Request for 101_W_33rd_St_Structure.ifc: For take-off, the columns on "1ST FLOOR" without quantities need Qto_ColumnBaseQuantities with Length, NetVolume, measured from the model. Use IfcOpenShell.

First a look at what the model holds.

```python
import ifcopenshell
import ifcopenshell.util.element
import ifcopenshell.util.unit

model = ifcopenshell.open("101_W_33rd_St_Structure.ifc")
print(model.schema)
for unit_type in ("LENGTHUNIT", "AREAUNIT", "VOLUMEUNIT"):
    print(unit_type, ifcopenshell.util.unit.calculate_unit_scale(model, unit_type))
storey = next(s for s in model.by_type("IfcBuildingStorey") if s.Name == "1ST FLOOR")
columns = [e for e in ifcopenshell.util.element.get_decomposition(storey) if e.is_a("IfcColumn")]
for e in sorted(columns, key=lambda e: e.id()):
    print(e.id(), e.is_a(), e.Name, list(ifcopenshell.util.element.get_psets(e, qtos_only=True)), sep=" | ")
```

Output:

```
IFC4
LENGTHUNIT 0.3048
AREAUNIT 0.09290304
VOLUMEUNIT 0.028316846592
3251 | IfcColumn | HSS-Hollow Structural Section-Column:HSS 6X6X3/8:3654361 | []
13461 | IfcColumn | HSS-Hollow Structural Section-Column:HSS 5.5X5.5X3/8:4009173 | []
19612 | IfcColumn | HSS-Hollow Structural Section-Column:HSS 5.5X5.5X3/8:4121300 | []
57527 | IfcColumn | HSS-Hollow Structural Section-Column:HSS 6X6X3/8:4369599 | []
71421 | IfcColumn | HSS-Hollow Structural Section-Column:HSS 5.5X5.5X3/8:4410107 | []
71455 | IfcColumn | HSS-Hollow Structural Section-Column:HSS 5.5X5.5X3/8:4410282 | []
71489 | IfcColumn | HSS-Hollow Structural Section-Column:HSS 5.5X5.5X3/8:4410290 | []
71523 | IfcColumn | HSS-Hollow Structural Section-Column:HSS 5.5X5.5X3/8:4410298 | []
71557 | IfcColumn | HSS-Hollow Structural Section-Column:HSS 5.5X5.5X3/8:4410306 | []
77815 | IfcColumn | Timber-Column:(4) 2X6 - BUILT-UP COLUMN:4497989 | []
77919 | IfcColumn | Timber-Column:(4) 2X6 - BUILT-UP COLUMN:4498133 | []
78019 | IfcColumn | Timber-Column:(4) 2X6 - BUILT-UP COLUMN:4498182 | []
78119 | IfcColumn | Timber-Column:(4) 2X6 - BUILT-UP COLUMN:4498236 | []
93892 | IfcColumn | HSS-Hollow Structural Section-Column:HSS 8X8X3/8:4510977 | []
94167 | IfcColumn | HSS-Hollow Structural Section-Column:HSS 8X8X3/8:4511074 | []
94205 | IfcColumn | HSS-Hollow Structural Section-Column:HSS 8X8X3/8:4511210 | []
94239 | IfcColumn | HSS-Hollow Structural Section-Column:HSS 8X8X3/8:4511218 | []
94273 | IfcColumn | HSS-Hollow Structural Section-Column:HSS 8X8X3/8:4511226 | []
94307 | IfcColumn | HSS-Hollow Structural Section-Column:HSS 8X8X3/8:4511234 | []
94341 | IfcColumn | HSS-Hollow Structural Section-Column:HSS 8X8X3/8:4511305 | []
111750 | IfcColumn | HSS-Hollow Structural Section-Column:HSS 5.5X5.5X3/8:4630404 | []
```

```python
import ifcopenshell
import ifcopenshell.api.pset
import ifcopenshell.geom
import ifcopenshell.util.element
import ifcopenshell.util.shape
import ifcopenshell.util.unit

model = ifcopenshell.open("101_W_33rd_St_Structure.ifc")
unit_scale = ifcopenshell.util.unit.calculate_unit_scale(model)
volume_scale = ifcopenshell.util.unit.calculate_unit_scale(model, "VOLUMEUNIT")
settings = ifcopenshell.geom.settings()

storey = next(s for s in model.by_type("IfcBuildingStorey") if s.Name == "1ST FLOOR")
columns = [e for e in ifcopenshell.util.element.get_decomposition(storey) if e.is_a("IfcColumn")]

for e in sorted(columns, key=lambda e: e.id()):
    if ifcopenshell.util.element.get_psets(e, qtos_only=True, should_inherit=False):
        continue
    # Geometry comes back in metres, in the element's own axes.
    shape = ifcopenshell.geom.create_shape(settings, e)
    values = {
        "Length": ifcopenshell.util.shape.get_z(shape.geometry) / unit_scale,
        "NetVolume": ifcopenshell.util.shape.get_volume(shape.geometry) / volume_scale,
    }
    qto = ifcopenshell.api.pset.add_qto(model, product=e, name="Qto_ColumnBaseQuantities")
    ifcopenshell.api.pset.edit_qto(model, qto=qto, properties=values)
    print(e.id(), {k: round(v, 3) for k, v in values.items()})

model.write("101_W_33rd_St_Structure_updated.ifc")
```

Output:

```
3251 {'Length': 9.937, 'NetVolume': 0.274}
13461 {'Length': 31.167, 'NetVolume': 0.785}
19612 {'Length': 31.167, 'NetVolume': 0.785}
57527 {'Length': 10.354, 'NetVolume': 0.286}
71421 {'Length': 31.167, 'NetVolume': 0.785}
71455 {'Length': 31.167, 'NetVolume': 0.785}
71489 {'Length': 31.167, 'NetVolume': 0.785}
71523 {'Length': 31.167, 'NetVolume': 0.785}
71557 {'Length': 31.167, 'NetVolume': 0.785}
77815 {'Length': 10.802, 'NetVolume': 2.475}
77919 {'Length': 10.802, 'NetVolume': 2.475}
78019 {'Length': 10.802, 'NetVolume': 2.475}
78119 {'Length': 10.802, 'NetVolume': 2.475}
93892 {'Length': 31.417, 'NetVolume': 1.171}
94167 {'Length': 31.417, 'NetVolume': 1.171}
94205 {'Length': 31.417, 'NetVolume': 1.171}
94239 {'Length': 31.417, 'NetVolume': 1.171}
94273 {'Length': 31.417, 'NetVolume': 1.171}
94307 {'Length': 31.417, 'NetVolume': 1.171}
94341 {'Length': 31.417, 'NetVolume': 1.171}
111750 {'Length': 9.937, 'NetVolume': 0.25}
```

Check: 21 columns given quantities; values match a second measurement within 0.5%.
